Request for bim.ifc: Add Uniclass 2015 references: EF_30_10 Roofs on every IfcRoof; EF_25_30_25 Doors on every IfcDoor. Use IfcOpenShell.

First a look at what the model holds.

```python
import ifcopenshell

model = ifcopenshell.open("bim.ifc")
print(model.schema)
print("classifications:", [c.Name for c in model.by_type("IfcClassification")])
for ifc_class in ("IfcDoor", "IfcRoof", "IfcStair", "IfcWall", "IfcWindow"):
    print(ifc_class, len(model.by_type(ifc_class)))
```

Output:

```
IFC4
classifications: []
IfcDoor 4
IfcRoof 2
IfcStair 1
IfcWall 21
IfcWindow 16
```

```python
import ifcopenshell
import ifcopenshell.api.classification

model = ifcopenshell.open("bim.ifc")

system = ifcopenshell.api.classification.add_classification(model, classification="Uniclass 2015")

codes = {
    "IfcRoof": ("EF_30_10", "Roofs"),
    "IfcDoor": ("EF_25_30_25", "Doors"),
}
for ifc_class, (code, name) in codes.items():
    products = model.by_type(ifc_class)
    ifcopenshell.api.classification.add_reference(
        model, products=products, classification=system, identification=code, name=name
    )
    print(code, len(products))

model.write("bim_rev.ifc")
```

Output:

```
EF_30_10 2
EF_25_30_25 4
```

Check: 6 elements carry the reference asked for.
